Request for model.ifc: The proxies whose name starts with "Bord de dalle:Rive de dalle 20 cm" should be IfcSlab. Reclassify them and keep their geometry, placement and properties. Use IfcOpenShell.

First a look at what the model holds.

```python
import re

import ifcopenshell

model = ifcopenshell.open("model.ifc")
print(model.schema)
seen = {}
for e in model.by_type("IfcBuildingElementProxy"):
    name = re.sub(r":\d+(:\d+)?$", "", e.Name or "")  # drop the element id that some exporters append
    seen[name] = seen.get(name, 0) + 1
for name, count in sorted(seen.items()):
    print(count, "x", name)
```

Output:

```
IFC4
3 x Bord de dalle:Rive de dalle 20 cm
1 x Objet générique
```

```python
import ifcopenshell
import ifcopenshell.api.root

model = ifcopenshell.open("model.ifc")

proxies = [e.id() for e in model.by_type("IfcBuildingElementProxy") if (e.Name or "").startswith("Bord de dalle:Rive de dalle 20 cm")]
for step_id in proxies:
    proxy = model.by_id(step_id)
    # Reclassifying a typed element also reclassifies its type and the type's other occurrences.
    if proxy.is_a("IfcBuildingElementProxy"):
        ifcopenshell.api.root.reassign_class(model, product=proxy, ifc_class="IfcSlab", predefined_type="FLOOR")

print(sum(model.by_id(i).is_a("IfcSlab") for i in proxies), "reclassified")

model.write("model_edited.ifc")
```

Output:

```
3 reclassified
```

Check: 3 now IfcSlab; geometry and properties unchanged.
